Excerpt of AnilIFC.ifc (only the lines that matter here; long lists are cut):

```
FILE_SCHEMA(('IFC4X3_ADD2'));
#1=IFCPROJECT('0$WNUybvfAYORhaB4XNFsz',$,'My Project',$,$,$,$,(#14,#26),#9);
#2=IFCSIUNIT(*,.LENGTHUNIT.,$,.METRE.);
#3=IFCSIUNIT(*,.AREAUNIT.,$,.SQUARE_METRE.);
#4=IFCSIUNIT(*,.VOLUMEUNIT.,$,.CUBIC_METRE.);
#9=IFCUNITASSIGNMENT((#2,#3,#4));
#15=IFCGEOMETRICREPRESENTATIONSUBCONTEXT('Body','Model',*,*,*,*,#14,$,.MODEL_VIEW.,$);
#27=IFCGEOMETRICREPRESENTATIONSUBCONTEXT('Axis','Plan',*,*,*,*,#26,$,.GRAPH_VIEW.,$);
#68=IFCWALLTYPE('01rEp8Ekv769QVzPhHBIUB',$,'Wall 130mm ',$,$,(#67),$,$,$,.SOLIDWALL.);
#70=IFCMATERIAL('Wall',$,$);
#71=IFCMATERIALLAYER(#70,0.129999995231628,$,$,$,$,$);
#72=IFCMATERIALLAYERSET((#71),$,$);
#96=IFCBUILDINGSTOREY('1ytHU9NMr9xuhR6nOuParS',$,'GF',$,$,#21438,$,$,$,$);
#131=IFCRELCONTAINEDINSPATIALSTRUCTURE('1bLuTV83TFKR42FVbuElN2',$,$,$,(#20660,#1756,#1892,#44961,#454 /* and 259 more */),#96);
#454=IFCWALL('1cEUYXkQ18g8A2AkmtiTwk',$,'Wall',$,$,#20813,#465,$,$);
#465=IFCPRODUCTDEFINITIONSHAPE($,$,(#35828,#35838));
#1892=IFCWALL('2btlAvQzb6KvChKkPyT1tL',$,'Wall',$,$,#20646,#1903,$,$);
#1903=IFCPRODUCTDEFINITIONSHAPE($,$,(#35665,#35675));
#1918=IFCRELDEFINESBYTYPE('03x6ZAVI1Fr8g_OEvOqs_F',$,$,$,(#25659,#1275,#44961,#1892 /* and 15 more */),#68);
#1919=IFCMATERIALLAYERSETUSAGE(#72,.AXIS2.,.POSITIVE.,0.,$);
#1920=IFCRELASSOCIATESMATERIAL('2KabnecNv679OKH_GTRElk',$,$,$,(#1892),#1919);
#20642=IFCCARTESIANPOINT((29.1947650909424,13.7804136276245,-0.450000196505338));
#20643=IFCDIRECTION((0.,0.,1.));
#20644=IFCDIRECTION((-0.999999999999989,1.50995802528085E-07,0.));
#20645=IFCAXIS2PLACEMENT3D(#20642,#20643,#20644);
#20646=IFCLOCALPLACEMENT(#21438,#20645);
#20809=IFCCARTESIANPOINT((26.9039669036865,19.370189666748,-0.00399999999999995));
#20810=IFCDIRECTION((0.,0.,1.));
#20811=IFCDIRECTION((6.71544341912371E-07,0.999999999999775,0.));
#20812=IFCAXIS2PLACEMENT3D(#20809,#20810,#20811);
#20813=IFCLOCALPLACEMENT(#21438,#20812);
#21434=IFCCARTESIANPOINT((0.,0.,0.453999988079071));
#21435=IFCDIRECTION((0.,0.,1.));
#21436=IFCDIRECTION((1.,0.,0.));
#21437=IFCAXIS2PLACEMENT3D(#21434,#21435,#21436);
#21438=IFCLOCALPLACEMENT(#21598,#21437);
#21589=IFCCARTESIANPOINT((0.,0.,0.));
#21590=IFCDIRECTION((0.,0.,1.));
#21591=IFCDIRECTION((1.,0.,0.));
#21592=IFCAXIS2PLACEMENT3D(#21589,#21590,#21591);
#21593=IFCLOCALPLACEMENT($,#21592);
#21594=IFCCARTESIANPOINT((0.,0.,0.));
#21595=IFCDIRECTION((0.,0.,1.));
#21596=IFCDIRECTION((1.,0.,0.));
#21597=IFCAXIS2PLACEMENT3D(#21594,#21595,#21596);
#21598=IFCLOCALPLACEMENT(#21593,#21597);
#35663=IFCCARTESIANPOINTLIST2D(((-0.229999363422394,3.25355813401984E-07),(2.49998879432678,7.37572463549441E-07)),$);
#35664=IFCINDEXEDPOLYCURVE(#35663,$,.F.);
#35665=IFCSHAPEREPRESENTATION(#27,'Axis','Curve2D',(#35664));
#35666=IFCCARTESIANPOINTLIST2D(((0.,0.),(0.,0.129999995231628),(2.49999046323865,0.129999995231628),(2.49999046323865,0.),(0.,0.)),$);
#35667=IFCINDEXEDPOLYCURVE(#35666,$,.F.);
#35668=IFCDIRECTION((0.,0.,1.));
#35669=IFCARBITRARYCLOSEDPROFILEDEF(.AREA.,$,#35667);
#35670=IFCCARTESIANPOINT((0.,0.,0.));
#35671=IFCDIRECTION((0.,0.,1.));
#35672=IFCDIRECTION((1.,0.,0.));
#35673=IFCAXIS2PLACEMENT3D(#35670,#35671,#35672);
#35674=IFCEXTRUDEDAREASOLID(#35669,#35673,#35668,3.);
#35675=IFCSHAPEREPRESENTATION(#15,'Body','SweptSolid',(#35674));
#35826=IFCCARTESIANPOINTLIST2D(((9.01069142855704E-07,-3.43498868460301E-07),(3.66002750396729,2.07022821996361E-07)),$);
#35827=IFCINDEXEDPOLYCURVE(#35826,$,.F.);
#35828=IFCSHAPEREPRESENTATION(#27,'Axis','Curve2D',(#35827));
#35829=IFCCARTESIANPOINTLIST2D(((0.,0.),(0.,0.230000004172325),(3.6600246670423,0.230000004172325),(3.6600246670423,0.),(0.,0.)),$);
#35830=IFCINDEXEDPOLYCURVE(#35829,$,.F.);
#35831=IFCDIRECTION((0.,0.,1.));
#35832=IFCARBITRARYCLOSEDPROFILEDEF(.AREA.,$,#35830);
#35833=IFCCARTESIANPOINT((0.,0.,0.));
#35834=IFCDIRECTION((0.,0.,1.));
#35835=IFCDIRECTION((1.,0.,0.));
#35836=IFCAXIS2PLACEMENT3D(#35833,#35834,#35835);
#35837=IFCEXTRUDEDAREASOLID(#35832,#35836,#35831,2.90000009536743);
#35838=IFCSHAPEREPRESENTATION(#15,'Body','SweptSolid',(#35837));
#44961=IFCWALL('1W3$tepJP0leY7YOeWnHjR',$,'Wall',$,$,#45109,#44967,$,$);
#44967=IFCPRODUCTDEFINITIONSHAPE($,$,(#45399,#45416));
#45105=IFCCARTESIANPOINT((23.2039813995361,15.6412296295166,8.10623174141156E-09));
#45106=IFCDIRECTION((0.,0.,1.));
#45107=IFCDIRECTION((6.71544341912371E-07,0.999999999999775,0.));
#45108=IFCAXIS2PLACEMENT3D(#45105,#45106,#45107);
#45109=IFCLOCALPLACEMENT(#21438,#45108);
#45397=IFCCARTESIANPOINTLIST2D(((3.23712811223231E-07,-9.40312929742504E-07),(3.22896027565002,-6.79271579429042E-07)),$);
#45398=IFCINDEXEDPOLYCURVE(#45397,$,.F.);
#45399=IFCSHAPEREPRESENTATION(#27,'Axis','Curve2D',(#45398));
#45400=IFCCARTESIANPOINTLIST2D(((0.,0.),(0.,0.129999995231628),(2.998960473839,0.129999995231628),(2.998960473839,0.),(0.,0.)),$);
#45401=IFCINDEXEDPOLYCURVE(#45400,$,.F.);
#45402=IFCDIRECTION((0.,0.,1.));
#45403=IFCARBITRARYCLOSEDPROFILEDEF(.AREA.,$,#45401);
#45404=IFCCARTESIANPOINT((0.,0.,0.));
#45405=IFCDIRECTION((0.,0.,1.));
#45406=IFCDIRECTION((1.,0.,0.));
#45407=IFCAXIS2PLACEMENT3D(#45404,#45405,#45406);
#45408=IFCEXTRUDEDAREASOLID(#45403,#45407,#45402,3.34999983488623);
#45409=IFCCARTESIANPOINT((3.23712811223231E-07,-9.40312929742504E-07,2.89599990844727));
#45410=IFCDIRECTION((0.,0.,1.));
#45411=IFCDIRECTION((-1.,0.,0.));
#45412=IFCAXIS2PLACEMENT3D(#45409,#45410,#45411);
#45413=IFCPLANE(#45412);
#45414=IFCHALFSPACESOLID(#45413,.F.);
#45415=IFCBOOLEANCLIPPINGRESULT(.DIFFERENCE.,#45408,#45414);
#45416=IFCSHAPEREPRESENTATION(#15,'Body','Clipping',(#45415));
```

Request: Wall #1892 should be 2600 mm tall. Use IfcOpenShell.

```python
import ifcopenshell
import ifcopenshell.geom
import ifcopenshell.util.representation
import ifcopenshell.util.shape
import ifcopenshell.util.unit

model = ifcopenshell.open("AnilIFC.ifc")
unit_scale = ifcopenshell.util.unit.calculate_unit_scale(model)
settings = ifcopenshell.geom.settings()


def volume(element):
    """Net volume in cubic metres, openings subtracted."""
    shape = ifcopenshell.geom.create_shape(settings, element)
    return ifcopenshell.util.shape.get_volume(shape.geometry)


wall = model.by_guid("2btlAvQzb6KvChKkPyT1tL")
before = volume(wall)

body = ifcopenshell.util.representation.get_representation(wall, "Model", "Body")
solid = body.Items[0]
old_height = solid.Depth
solid.Depth = 2.6 / unit_scale
after = volume(wall)

print(f"height {old_height:g} -> {solid.Depth:g}, volume {before:.3f} -> {after:.3f} m3")

model.write("AnilIFC_v2.ifc")
```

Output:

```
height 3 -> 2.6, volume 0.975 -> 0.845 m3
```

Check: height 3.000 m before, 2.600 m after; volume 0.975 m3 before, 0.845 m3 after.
